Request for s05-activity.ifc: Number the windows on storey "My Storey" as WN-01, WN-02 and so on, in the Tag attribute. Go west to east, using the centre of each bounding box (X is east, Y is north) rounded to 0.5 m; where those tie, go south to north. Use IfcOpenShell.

First a look at what the model holds.

```python
import ifcopenshell
import ifcopenshell.util.element
import ifcopenshell.util.placement

model = ifcopenshell.open("s05-activity.ifc")
print(model.schema)
storey = next(s for s in model.by_type("IfcBuildingStorey") if s.Name == "My Storey")
windows = [e for e in ifcopenshell.util.element.get_decomposition(storey) if e.is_a("IfcWindow")]
for e in sorted(windows, key=lambda e: e.id()):
    origin = ifcopenshell.util.placement.get_local_placement(e.ObjectPlacement)[:3, 3]
    print(e.id(), e.Tag, e.Name, origin.round(2) + 0.0, sep=" | ")
```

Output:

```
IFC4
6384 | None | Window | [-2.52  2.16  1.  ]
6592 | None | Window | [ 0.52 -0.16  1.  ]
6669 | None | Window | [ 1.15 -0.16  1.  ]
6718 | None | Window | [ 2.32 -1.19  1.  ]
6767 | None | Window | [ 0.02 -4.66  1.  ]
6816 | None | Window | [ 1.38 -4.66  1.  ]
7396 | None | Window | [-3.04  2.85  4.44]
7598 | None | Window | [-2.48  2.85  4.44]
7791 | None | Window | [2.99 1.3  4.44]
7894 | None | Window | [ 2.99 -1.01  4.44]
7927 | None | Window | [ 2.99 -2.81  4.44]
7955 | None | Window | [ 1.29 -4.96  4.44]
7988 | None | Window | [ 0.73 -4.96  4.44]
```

```python
import ifcopenshell
import ifcopenshell.geom
import ifcopenshell.util.element
import ifcopenshell.util.shape

model = ifcopenshell.open("s05-activity.ifc")
settings = ifcopenshell.geom.settings()
settings.set("use-world-coords", True)


def centre(element):
    shape = ifcopenshell.geom.create_shape(settings, element)
    return ifcopenshell.util.shape.get_bbox_centroid(shape.geometry)


storey = next(s for s in model.by_type("IfcBuildingStorey") if s.Name == "My Storey")
windows = [e for e in ifcopenshell.util.element.get_decomposition(storey) if e.is_a("IfcWindow")]

# Insertion points can sit at a corner or the storey origin, so sort by the geometry (in metres).
centres = {e: centre(e) for e in windows}
windows.sort(key=lambda e: (round(centres[e][0] / 0.5), centres[e][1]))

for i, e in enumerate(windows, start=1):
    number = f"WN-{i:02d}"
    e.Tag = number
    print(e.id(), number)

model.write("s05-activity_updated.ifc")
```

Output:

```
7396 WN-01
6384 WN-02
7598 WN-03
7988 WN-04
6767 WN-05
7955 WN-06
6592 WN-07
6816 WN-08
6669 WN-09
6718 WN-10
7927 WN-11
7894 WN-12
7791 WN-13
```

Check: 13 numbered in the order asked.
